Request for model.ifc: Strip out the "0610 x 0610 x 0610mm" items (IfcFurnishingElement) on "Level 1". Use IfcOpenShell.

First a look at what the model holds.

```python
import ifcopenshell
import ifcopenshell.util.element

model = ifcopenshell.open("model.ifc")
print(model.schema)
storey = next(s for s in model.by_type("IfcBuildingStorey") if s.Name == "Level 1")
furniture = [e for e in ifcopenshell.util.element.get_decomposition(storey) if e.is_a("IfcFurnishingElement")]
seen = {}
for e in furniture:
    element_type = ifcopenshell.util.element.get_type(e)
    name = element_type.Name if element_type not in (None, e) else None
    seen[name] = seen.get(name, 0) + 1
for name, count in sorted(seen.items(), key=str):
    print(count, "x", name)
```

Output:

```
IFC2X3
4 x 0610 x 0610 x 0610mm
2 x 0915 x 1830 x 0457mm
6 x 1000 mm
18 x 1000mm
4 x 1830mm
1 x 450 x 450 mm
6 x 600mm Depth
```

```python
import ifcopenshell
import ifcopenshell.api.root
import ifcopenshell.util.element

model = ifcopenshell.open("model.ifc")

storey = next(s for s in model.by_type("IfcBuildingStorey") if s.Name == "Level 1")
furniture = [e for e in ifcopenshell.util.element.get_decomposition(storey) if e.is_a("IfcFurnishingElement")]
targets = [e for e in furniture if (t := ifcopenshell.util.element.get_type(e)) not in (None, e) and t.Name == "0610 x 0610 x 0610mm"]

for e in targets:
    ifcopenshell.api.root.remove_product(model, product=e)
print(len(targets), "removed")

model.write("model_rev.ifc")
```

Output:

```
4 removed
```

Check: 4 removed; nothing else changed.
